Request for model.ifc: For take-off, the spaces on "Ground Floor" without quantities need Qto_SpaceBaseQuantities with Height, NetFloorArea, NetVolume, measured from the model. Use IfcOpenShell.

First a look at what the model holds.

```python
import ifcopenshell
import ifcopenshell.util.element
import ifcopenshell.util.unit

model = ifcopenshell.open("model.ifc")
print(model.schema)
for unit_type in ("LENGTHUNIT", "AREAUNIT", "VOLUMEUNIT"):
    print(unit_type, ifcopenshell.util.unit.calculate_unit_scale(model, unit_type))
storey = next(s for s in model.by_type("IfcBuildingStorey") if s.Name == "Ground Floor")
spaces = [e for e in ifcopenshell.util.element.get_decomposition(storey) if e.is_a("IfcSpace")]
for e in sorted(spaces, key=lambda e: e.id()):
    print(e.id(), e.is_a(), e.Name, list(ifcopenshell.util.element.get_psets(e, qtos_only=True)), sep=" | ")
```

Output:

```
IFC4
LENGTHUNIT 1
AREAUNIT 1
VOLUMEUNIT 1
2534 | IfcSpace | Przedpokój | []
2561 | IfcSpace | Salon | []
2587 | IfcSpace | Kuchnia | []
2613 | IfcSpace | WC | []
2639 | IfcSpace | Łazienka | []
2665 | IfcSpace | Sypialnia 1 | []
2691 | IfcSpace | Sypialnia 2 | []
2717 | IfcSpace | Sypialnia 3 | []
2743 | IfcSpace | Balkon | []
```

```python
import ifcopenshell
import ifcopenshell.api.pset
import ifcopenshell.geom
import ifcopenshell.util.element
import ifcopenshell.util.shape
import ifcopenshell.util.unit

model = ifcopenshell.open("model.ifc")
unit_scale = ifcopenshell.util.unit.calculate_unit_scale(model)
area_scale = ifcopenshell.util.unit.calculate_unit_scale(model, "AREAUNIT")
volume_scale = ifcopenshell.util.unit.calculate_unit_scale(model, "VOLUMEUNIT")
settings = ifcopenshell.geom.settings()

storey = next(s for s in model.by_type("IfcBuildingStorey") if s.Name == "Ground Floor")
spaces = [e for e in ifcopenshell.util.element.get_decomposition(storey) if e.is_a("IfcSpace")]

for e in sorted(spaces, key=lambda e: e.id()):
    if ifcopenshell.util.element.get_psets(e, qtos_only=True, should_inherit=False):
        continue
    # Geometry comes back in metres, in the element's own axes.
    shape = ifcopenshell.geom.create_shape(settings, e)
    values = {
        "Height": ifcopenshell.util.shape.get_z(shape.geometry) / unit_scale,
        "NetFloorArea": ifcopenshell.util.shape.get_footprint_area(shape.geometry) / area_scale,
        "NetVolume": ifcopenshell.util.shape.get_volume(shape.geometry) / volume_scale,
    }
    qto = ifcopenshell.api.pset.add_qto(model, product=e, name="Qto_SpaceBaseQuantities")
    ifcopenshell.api.pset.edit_qto(model, qto=qto, properties=values)
    print(e.id(), {k: round(v, 3) for k, v in values.items()})

model.write("model_rev.ifc")
```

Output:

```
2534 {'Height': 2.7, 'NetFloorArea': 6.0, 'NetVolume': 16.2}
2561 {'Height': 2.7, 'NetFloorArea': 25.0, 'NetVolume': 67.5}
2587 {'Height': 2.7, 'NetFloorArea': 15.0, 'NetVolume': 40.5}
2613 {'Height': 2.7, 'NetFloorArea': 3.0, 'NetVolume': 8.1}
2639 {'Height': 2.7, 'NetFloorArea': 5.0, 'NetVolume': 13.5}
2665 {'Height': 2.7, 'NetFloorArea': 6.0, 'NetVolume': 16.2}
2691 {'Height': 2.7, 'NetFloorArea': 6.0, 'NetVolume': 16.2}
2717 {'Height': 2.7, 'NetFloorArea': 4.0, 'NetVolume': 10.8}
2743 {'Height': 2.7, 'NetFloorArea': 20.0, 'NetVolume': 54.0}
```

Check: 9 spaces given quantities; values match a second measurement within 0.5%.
